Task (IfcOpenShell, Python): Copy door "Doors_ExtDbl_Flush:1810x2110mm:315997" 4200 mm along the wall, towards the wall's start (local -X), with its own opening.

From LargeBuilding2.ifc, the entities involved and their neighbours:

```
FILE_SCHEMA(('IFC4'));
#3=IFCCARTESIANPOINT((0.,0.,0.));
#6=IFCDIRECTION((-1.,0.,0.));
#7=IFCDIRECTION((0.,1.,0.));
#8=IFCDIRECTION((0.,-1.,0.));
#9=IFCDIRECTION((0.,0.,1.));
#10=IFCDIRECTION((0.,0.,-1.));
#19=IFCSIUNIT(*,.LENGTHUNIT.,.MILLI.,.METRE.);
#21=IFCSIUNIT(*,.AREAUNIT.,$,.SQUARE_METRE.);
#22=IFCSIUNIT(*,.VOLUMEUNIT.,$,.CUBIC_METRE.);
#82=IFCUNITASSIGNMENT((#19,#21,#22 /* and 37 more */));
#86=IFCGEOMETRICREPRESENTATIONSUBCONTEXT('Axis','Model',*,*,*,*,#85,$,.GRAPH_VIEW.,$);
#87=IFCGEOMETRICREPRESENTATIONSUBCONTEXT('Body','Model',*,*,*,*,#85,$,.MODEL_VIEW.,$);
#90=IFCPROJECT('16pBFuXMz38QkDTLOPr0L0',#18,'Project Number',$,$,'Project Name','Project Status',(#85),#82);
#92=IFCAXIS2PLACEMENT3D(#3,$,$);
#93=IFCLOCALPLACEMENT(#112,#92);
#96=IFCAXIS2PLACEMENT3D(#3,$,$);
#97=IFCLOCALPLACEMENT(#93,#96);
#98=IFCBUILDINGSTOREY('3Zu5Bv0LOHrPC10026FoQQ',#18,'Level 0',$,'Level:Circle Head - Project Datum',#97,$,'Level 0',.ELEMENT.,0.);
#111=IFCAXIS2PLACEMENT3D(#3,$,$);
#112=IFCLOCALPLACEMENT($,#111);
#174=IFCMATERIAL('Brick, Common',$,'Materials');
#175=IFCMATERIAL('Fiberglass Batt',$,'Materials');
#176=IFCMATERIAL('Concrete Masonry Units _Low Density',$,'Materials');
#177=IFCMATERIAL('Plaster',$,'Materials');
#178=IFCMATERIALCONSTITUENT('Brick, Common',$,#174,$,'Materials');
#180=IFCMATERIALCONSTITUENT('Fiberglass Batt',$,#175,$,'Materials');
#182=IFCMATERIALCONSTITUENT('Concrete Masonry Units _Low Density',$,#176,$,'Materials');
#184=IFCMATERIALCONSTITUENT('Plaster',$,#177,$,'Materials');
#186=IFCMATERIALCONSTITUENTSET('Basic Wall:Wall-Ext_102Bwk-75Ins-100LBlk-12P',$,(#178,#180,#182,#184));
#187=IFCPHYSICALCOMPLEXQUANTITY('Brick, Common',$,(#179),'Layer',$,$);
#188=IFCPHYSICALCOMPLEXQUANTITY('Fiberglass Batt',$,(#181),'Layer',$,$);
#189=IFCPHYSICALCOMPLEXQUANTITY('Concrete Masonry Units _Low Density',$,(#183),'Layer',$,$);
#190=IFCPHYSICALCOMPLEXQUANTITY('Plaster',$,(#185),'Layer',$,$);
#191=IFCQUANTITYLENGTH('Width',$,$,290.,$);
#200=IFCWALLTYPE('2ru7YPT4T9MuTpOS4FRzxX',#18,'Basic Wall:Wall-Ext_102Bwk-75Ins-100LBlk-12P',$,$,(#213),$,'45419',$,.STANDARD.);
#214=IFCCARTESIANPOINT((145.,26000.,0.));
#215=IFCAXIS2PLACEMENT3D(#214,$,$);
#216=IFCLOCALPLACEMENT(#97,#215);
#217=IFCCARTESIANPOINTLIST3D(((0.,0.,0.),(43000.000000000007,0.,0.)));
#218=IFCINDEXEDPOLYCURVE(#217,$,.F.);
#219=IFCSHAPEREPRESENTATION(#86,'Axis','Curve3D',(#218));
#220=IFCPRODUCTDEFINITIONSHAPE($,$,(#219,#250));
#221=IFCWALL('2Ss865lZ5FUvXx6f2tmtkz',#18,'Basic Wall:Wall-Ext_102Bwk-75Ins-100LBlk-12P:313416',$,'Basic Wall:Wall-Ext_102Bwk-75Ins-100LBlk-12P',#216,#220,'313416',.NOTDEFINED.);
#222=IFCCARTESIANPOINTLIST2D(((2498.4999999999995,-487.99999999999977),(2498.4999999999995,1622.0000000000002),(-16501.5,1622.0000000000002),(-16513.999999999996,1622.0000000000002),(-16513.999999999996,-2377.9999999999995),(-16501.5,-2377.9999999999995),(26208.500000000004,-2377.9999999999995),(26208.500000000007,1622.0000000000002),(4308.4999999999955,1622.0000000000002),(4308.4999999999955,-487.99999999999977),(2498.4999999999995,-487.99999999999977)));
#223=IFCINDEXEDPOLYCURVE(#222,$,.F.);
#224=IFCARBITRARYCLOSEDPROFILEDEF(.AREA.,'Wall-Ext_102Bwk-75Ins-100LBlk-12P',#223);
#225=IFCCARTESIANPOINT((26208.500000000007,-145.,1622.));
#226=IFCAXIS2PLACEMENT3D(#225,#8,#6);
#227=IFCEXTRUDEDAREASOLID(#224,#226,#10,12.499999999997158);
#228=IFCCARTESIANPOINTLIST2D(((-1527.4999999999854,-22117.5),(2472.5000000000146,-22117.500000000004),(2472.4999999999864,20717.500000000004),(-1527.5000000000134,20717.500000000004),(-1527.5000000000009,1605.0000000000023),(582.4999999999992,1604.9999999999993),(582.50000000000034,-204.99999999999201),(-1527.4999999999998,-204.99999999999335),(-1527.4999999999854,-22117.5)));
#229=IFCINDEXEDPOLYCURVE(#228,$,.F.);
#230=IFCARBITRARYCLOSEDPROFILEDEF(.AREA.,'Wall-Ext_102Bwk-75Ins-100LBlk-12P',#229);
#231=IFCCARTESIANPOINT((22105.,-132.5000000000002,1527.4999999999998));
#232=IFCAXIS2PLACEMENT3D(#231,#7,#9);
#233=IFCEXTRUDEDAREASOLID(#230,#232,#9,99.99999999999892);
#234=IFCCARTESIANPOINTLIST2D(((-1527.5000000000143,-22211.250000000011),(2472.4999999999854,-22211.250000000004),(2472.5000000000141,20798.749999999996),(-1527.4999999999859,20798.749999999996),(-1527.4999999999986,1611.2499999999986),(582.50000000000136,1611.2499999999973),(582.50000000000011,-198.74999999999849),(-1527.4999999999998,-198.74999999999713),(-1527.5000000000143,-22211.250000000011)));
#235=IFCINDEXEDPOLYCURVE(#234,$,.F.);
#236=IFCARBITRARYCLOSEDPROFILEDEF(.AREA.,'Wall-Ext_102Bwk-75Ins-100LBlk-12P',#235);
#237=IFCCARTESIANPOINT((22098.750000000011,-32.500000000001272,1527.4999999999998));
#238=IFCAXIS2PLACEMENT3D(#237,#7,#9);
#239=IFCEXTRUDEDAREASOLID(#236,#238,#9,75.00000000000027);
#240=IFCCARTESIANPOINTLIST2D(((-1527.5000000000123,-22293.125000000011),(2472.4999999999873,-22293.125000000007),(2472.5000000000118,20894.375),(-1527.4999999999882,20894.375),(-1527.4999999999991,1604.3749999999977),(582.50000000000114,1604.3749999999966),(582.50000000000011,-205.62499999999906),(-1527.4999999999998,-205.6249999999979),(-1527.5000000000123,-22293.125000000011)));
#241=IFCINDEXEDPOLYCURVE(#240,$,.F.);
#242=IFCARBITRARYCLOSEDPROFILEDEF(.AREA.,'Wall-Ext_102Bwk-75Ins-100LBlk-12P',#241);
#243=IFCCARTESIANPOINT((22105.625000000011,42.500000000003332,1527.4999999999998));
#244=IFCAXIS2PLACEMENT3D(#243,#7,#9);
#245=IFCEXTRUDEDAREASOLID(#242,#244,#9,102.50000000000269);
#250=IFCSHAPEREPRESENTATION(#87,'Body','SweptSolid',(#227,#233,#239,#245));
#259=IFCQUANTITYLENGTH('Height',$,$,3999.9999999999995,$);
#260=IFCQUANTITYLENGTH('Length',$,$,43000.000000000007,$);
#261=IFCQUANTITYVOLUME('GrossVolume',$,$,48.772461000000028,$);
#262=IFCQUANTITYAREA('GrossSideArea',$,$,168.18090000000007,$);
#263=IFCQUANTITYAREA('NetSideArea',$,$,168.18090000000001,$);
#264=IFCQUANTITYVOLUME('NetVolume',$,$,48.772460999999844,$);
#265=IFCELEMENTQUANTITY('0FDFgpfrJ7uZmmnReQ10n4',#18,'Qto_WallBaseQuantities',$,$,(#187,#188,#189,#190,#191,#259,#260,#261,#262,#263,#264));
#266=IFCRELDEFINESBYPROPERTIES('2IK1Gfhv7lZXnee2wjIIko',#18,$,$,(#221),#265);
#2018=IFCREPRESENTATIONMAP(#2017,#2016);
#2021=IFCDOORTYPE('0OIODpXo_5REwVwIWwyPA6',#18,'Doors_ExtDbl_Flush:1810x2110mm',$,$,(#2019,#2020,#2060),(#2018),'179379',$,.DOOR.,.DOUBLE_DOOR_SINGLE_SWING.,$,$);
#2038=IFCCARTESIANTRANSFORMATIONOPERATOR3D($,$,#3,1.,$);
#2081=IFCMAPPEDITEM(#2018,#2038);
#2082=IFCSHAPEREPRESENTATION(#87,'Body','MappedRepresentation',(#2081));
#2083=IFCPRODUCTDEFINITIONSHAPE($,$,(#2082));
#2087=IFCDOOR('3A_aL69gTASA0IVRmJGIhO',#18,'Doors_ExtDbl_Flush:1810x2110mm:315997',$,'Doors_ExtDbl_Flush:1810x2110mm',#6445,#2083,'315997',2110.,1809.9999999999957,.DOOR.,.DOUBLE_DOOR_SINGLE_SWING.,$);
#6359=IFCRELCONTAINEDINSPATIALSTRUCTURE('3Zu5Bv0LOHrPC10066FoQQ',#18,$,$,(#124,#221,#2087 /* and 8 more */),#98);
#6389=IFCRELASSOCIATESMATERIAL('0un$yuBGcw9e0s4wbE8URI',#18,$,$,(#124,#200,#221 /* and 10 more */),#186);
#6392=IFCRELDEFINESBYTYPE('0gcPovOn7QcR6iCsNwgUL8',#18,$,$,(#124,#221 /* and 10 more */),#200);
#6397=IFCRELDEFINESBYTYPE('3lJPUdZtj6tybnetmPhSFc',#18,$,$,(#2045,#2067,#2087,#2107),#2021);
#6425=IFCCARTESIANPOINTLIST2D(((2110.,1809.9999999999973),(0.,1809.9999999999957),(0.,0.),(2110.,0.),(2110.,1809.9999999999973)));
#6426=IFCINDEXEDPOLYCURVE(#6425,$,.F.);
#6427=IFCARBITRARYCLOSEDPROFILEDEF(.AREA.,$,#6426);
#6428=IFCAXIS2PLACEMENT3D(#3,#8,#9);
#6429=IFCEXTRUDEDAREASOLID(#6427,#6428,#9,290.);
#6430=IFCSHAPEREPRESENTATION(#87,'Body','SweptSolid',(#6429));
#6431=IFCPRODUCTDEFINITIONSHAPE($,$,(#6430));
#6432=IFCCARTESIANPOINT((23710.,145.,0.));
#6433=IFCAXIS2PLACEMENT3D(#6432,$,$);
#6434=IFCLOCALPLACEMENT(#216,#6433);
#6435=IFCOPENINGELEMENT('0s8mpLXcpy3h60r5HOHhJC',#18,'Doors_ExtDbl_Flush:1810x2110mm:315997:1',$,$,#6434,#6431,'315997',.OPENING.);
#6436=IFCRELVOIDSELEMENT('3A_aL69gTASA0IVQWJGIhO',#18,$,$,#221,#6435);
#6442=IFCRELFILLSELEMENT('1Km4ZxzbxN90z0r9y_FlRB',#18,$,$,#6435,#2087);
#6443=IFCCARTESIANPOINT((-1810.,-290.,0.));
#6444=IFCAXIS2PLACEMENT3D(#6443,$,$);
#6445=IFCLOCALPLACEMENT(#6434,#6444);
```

```python
import ifcopenshell
import ifcopenshell.api.feature
import ifcopenshell.api.geometry
import ifcopenshell.api.pset
import ifcopenshell.api.root
import ifcopenshell.geom
import ifcopenshell.util.element
import ifcopenshell.util.placement
import ifcopenshell.util.shape
import ifcopenshell.util.unit

model = ifcopenshell.open("LargeBuilding2.ifc")
unit_scale = ifcopenshell.util.unit.calculate_unit_scale(model)
area_scale = ifcopenshell.util.unit.calculate_unit_scale(model, "AREAUNIT")
volume_scale = ifcopenshell.util.unit.calculate_unit_scale(model, "VOLUMEUNIT")
settings = ifcopenshell.geom.settings()


def volume(element):
    """Net volume in cubic metres, openings subtracted."""
    shape = ifcopenshell.geom.create_shape(settings, element)
    return ifcopenshell.util.shape.get_volume(shape.geometry)


def reuse_history(source, copy):
    """copy_class also copies each property set's owner history, people and application; keep the originals."""
    for rel in copy.IsDefinedBy:
        if rel.is_a("IfcRelDefinesByProperties") and (history := rel.RelatingPropertyDefinition.OwnerHistory):
            rel.RelatingPropertyDefinition.OwnerHistory = source.OwnerHistory
            ifcopenshell.util.element.remove_deep2(model, history)


door = model.by_id(2087)
opening = door.FillsVoids[0].RelatingOpeningElement
wall = opening.VoidsElements[0].RelatingBuildingElement
before = volume(wall)
shift = ifcopenshell.util.placement.get_local_placement(wall.ObjectPlacement)[:3, 0] * -4.2 / unit_scale

# copy_class copies the void relationship, type, container and properties, but no geometry.
new_opening = ifcopenshell.api.root.copy_class(model, product=opening)
new_opening.Representation = ifcopenshell.util.element.copy_deep(
    model, opening.Representation, exclude=["IfcGeometricRepresentationContext", "IfcRepresentationMap"]
)
new_opening.Name = "Doors_ExtDbl_Flush:1810x2110mm"
new_opening.Tag = None
reuse_history(opening, new_opening)
new_door = ifcopenshell.api.root.copy_class(model, product=door)
new_door.Representation = ifcopenshell.util.element.copy_deep(
    model, door.Representation, exclude=["IfcGeometricRepresentationContext", "IfcRepresentationMap"]
)
new_door.Name = "Doors_ExtDbl_Flush:1810x2110mm"
new_door.Tag = None
reuse_history(door, new_door)
ifcopenshell.api.feature.add_filling(model, opening=new_opening, element=new_door)

for old, new in ((opening, new_opening), (door, new_door)):
    matrix = ifcopenshell.util.placement.get_local_placement(old.ObjectPlacement)
    matrix[:3, 3] += shift
    ifcopenshell.api.geometry.edit_object_placement(model, product=new, matrix=matrix, is_si=False)

after = volume(wall)
thickness = 0.29  # wall thickness in metres

# Update the wall's stored quantities.
qto = model.by_id(ifcopenshell.util.element.get_pset(wall, "Qto_WallBaseQuantities", should_inherit=False)["id"])
ifcopenshell.api.pset.edit_qto(model, qto=qto, properties={
    "NetSideArea": after / thickness / area_scale,
    "NetVolume": after / volume_scale,
})

print(f"wall volume {before:.3f} -> {after:.3f} m3")

model.write("LargeBuilding2_updated.ifc")
```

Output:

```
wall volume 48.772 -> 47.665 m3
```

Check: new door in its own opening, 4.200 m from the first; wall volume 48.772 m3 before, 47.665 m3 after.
